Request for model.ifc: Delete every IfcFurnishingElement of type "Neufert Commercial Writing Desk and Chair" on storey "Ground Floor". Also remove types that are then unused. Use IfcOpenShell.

First a look at what the model holds.

```python
import ifcopenshell
import ifcopenshell.util.element

model = ifcopenshell.open("model.ifc")
print(model.schema)
storey = next(s for s in model.by_type("IfcBuildingStorey") if s.Name == "Ground Floor")
furniture = [e for e in ifcopenshell.util.element.get_decomposition(storey) if e.is_a("IfcFurnishingElement")]
seen = {}
for e in furniture:
    element_type = ifcopenshell.util.element.get_type(e)
    name = element_type.Name if element_type not in (None, e) else None
    seen[name] = seen.get(name, 0) + 1
for name, count in sorted(seen.items(), key=str):
    print(count, "x", name)
```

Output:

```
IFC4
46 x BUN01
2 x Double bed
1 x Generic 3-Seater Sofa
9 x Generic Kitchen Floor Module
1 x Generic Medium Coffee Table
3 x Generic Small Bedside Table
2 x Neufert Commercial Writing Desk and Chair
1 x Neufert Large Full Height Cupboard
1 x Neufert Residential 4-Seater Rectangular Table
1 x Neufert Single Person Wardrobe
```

```python
import ifcopenshell
import ifcopenshell.api.root
import ifcopenshell.util.element

model = ifcopenshell.open("model.ifc")

storey = next(s for s in model.by_type("IfcBuildingStorey") if s.Name == "Ground Floor")
furniture = [e for e in ifcopenshell.util.element.get_decomposition(storey) if e.is_a("IfcFurnishingElement")]
targets = [e for e in furniture if (t := ifcopenshell.util.element.get_type(e)) not in (None, e) and t.Name == "Neufert Commercial Writing Desk and Chair"]
types = {ifcopenshell.util.element.get_type(e) for e in targets} - {None, *targets}

for e in targets:
    ifcopenshell.api.root.remove_product(model, product=e)
print(len(targets), "removed")

unused = [t for t in types if not ifcopenshell.util.element.get_types(t)]
for t in unused:
    ifcopenshell.api.root.remove_product(model, product=t)
print(len(unused), "unused types removed")

model.write("model_edited.ifc")
```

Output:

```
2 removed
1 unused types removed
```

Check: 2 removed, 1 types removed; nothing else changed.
